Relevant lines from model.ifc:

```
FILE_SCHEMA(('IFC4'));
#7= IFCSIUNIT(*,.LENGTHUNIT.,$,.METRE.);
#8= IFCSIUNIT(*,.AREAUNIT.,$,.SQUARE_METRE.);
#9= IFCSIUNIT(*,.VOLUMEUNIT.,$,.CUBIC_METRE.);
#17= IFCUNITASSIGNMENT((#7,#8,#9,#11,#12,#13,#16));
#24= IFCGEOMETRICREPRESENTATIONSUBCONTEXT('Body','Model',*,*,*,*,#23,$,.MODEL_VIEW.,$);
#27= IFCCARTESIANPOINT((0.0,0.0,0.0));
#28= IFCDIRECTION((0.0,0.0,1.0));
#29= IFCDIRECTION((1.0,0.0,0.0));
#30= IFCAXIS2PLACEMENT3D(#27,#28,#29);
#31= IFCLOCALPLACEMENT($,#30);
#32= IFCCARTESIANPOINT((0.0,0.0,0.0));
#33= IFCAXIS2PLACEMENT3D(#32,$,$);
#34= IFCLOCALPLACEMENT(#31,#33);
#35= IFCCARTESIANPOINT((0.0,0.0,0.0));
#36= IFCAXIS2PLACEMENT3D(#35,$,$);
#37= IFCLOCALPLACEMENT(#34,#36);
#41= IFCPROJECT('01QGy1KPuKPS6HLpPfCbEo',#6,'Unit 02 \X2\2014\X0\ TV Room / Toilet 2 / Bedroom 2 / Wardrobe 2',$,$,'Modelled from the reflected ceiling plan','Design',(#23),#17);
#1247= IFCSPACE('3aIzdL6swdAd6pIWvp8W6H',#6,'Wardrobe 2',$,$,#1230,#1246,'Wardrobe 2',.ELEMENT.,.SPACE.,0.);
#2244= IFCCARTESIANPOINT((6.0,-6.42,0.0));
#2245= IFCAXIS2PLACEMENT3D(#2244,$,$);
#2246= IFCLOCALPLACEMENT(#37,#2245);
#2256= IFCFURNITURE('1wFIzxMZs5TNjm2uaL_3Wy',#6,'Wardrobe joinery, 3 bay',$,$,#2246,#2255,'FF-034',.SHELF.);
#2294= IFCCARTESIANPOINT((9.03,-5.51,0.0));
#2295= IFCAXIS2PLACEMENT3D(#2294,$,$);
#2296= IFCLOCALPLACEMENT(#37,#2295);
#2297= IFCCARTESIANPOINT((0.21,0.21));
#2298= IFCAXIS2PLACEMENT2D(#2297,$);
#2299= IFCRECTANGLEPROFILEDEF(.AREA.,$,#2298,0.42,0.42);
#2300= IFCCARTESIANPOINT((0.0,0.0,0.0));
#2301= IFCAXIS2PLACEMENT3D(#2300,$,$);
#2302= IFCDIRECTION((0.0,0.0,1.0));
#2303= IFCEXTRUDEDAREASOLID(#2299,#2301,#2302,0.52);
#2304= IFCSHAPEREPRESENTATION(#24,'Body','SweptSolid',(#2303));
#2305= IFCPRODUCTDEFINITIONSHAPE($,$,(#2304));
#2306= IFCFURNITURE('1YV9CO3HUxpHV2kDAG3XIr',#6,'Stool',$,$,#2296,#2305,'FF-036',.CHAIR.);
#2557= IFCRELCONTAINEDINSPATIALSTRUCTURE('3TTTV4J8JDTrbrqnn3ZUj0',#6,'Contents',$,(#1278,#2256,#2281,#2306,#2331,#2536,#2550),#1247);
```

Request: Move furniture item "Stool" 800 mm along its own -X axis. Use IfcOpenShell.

```python
import ifcopenshell
import ifcopenshell.api.geometry
import ifcopenshell.util.placement
import ifcopenshell.util.unit

model = ifcopenshell.open("model.ifc")
unit_scale = ifcopenshell.util.unit.calculate_unit_scale(model)

item = model.by_guid("1YV9CO3HUxpHV2kDAG3XIr")
matrix = ifcopenshell.util.placement.get_local_placement(item.ObjectPlacement)
matrix[:3, 3] -= matrix[:3, 0] * 0.8 / unit_scale
ifcopenshell.api.geometry.edit_object_placement(model, product=item, matrix=matrix, is_si=False)

print(ifcopenshell.util.placement.get_local_placement(item.ObjectPlacement).round(3) + 0.0)

model.write("model_rev.ifc")
```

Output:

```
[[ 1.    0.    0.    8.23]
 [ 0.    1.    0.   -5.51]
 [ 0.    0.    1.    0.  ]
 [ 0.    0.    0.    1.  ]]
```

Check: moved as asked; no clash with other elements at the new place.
